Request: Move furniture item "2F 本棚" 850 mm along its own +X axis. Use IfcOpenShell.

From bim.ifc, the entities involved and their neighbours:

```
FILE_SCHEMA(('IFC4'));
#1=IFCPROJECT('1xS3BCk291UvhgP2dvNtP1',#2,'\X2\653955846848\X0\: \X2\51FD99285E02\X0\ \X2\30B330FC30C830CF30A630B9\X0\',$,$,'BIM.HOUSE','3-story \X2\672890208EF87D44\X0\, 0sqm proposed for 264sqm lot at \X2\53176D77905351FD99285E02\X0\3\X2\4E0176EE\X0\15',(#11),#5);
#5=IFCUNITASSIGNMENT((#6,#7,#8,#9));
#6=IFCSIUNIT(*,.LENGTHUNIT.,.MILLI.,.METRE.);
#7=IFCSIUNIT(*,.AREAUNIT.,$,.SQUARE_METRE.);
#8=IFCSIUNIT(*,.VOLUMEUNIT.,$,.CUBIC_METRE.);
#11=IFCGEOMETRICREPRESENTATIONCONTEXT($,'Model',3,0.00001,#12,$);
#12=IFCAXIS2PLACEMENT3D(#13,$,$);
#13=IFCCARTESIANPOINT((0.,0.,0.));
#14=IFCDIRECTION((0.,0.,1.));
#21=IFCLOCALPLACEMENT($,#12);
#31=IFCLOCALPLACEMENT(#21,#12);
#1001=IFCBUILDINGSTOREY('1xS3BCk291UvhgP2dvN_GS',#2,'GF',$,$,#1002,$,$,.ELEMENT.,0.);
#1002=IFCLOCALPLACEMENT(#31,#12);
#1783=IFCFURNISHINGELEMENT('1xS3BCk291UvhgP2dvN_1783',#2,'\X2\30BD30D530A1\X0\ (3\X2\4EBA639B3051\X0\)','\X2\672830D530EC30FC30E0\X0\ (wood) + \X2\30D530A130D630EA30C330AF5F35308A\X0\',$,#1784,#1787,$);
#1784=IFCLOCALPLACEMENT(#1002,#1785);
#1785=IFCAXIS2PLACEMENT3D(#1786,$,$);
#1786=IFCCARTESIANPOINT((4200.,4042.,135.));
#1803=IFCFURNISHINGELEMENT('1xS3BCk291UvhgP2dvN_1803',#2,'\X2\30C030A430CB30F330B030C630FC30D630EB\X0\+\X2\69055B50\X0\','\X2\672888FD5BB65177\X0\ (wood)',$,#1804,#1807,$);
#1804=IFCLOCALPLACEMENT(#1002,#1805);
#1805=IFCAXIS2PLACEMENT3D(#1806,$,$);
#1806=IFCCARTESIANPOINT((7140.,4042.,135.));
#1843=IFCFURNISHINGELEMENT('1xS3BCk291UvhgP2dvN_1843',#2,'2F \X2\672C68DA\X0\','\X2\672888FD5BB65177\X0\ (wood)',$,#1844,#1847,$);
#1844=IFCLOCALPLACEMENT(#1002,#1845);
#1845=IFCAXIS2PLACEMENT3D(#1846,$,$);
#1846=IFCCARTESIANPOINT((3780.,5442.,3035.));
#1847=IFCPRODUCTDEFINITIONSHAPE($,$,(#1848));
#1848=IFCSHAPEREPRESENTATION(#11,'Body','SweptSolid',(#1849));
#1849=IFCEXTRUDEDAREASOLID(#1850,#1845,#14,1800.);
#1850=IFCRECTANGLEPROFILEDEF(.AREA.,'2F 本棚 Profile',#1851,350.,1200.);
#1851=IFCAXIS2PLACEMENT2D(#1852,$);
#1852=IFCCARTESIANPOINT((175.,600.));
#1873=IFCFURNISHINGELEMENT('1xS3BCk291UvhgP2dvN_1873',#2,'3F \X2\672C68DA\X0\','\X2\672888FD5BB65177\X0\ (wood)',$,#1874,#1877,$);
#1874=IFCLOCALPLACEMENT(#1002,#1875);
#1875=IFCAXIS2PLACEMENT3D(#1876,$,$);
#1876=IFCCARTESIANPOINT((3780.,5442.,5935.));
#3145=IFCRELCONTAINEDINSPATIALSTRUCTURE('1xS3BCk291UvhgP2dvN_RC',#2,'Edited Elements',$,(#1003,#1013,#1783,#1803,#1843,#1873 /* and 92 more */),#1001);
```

```python
import ifcopenshell
import ifcopenshell.api.geometry
import ifcopenshell.util.placement
import ifcopenshell.util.unit

model = ifcopenshell.open("bim.ifc")
unit_scale = ifcopenshell.util.unit.calculate_unit_scale(model)

item = model.by_guid("1xS3BCk291UvhgP2dvN_1843")
matrix = ifcopenshell.util.placement.get_local_placement(item.ObjectPlacement)
matrix[:3, 3] += matrix[:3, 0] * 0.85 / unit_scale
ifcopenshell.api.geometry.edit_object_placement(model, product=item, matrix=matrix, is_si=False)

print(ifcopenshell.util.placement.get_local_placement(item.ObjectPlacement).round(3) + 0.0)

model.write("bim_edited.ifc")
```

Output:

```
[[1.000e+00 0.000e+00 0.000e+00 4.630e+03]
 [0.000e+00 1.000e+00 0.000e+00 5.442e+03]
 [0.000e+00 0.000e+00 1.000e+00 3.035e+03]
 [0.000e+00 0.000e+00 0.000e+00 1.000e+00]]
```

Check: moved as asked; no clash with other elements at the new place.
